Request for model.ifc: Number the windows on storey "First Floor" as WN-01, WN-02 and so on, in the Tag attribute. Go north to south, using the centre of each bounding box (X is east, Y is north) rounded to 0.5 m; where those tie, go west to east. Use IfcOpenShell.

First a look at what the model holds.

```python
import ifcopenshell
import ifcopenshell.util.element
import ifcopenshell.util.placement

model = ifcopenshell.open("model.ifc")
print(model.schema)
storey = next(s for s in model.by_type("IfcBuildingStorey") if s.Name == "First Floor")
windows = [e for e in ifcopenshell.util.element.get_decomposition(storey) if e.is_a("IfcWindow")]
for e in sorted(windows, key=lambda e: e.id()):
    origin = ifcopenshell.util.placement.get_local_placement(e.ObjectPlacement)[:3, 3]
    print(e.id(), e.Tag, e.Name, origin.round(2) + 0.0, sep=" | ")
```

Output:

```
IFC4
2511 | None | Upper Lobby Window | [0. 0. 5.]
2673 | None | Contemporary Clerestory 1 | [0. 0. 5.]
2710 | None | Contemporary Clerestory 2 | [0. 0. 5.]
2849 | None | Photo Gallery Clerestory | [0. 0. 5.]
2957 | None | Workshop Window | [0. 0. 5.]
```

```python
import ifcopenshell
import ifcopenshell.geom
import ifcopenshell.util.element
import ifcopenshell.util.shape

model = ifcopenshell.open("model.ifc")
settings = ifcopenshell.geom.settings()
settings.set("use-world-coords", True)


def centre(element):
    shape = ifcopenshell.geom.create_shape(settings, element)
    return ifcopenshell.util.shape.get_bbox_centroid(shape.geometry)


storey = next(s for s in model.by_type("IfcBuildingStorey") if s.Name == "First Floor")
windows = [e for e in ifcopenshell.util.element.get_decomposition(storey) if e.is_a("IfcWindow")]

# Insertion points can sit at a corner or the storey origin, so sort by the geometry (in metres).
centres = {e: centre(e) for e in windows}
windows.sort(key=lambda e: (-round(centres[e][1] / 0.5), centres[e][0]))

for i, e in enumerate(windows, start=1):
    number = f"WN-{i:02d}"
    e.Tag = number
    print(e.id(), number)

model.write("model-out.ifc")
```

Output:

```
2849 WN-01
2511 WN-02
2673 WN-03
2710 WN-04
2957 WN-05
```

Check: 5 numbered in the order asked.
